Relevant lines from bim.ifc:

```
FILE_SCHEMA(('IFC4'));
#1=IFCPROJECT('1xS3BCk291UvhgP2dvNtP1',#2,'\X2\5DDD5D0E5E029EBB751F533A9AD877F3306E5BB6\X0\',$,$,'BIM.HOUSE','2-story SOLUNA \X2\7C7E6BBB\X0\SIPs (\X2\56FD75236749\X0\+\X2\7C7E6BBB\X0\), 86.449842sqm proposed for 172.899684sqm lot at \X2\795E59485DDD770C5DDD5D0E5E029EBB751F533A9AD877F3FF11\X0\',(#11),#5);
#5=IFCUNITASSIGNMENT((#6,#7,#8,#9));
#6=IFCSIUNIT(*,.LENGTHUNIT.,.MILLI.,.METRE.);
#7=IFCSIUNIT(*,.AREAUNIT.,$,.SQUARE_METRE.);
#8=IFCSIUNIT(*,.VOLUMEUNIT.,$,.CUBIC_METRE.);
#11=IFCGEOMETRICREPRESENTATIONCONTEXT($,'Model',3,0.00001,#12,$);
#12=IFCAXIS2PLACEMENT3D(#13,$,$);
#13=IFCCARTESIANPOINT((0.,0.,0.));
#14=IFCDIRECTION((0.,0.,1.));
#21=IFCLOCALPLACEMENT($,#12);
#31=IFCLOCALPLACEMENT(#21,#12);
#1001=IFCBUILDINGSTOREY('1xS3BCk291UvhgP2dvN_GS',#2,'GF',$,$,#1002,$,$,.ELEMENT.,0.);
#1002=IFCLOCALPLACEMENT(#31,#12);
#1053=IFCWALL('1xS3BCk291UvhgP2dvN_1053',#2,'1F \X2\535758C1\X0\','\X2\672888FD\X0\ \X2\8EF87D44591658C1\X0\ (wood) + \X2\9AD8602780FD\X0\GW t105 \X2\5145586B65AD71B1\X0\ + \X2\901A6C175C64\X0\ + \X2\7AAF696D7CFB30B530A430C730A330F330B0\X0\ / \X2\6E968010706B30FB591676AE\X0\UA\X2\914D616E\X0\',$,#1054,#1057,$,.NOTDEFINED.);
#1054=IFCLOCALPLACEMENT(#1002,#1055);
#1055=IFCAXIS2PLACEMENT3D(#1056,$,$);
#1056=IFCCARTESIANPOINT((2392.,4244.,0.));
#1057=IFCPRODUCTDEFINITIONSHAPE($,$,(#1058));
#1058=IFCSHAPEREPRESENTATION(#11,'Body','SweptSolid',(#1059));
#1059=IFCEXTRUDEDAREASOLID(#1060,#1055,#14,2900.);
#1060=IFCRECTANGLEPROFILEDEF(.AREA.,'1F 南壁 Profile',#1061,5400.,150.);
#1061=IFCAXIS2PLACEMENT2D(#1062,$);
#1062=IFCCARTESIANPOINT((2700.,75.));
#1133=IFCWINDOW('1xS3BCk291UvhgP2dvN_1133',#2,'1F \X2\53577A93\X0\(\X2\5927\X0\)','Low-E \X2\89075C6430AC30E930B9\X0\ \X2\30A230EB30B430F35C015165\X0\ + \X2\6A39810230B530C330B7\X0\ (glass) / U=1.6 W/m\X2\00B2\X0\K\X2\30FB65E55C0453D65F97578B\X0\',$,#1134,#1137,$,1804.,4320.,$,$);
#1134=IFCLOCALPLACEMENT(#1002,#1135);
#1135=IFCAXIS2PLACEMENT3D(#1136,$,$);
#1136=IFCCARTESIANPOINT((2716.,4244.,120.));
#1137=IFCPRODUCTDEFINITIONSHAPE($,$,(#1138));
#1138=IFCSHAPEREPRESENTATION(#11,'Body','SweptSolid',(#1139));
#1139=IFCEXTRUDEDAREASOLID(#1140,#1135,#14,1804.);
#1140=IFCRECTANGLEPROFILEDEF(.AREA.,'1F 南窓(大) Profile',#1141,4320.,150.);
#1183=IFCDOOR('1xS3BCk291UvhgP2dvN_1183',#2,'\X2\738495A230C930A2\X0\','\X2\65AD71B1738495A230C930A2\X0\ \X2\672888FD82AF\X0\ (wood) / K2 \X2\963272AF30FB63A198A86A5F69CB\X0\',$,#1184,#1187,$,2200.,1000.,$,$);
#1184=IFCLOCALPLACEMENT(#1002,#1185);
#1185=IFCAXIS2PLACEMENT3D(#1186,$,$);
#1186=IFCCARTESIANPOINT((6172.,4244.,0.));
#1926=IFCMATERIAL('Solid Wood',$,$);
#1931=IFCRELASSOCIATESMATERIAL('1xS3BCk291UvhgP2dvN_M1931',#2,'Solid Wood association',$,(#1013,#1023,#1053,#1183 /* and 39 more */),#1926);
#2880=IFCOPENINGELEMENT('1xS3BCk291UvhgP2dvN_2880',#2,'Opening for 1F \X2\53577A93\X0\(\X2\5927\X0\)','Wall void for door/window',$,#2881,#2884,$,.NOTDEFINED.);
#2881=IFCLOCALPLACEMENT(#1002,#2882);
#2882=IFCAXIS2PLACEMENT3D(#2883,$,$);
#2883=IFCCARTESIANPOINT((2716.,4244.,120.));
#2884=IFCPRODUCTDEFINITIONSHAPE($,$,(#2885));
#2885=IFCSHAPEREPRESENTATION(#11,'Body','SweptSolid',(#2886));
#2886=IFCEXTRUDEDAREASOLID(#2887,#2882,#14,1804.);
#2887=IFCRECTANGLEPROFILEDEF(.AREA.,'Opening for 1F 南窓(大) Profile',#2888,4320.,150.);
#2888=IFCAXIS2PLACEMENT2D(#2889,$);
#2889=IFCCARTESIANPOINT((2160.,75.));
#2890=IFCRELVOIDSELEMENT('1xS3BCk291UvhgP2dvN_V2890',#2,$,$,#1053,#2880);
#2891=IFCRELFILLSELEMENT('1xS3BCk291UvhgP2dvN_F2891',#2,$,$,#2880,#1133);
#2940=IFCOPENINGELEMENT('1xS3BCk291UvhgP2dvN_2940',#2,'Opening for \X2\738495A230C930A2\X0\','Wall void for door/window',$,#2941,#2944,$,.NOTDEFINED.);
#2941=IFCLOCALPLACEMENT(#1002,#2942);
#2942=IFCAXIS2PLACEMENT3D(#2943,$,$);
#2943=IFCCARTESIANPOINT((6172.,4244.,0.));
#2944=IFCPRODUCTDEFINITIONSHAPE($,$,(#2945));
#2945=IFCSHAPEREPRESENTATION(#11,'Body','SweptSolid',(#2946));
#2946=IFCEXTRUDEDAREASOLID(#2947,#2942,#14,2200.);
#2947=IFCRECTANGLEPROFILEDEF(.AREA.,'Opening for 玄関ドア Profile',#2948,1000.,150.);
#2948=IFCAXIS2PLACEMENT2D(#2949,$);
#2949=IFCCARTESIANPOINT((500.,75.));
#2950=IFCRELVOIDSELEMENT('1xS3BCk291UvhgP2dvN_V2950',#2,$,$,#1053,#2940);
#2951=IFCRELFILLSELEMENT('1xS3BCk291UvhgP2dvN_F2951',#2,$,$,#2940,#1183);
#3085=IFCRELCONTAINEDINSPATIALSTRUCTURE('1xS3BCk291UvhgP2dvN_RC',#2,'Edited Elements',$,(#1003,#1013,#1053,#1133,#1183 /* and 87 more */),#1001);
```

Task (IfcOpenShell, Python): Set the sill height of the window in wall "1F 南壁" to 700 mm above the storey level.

```python
import numpy as np
import ifcopenshell
import ifcopenshell.api.geometry
import ifcopenshell.geom
import ifcopenshell.util.element
import ifcopenshell.util.placement
import ifcopenshell.util.shape
import ifcopenshell.util.unit

model = ifcopenshell.open("bim.ifc")
unit_scale = ifcopenshell.util.unit.calculate_unit_scale(model)

window = model.by_id(1133)
opening = window.FillsVoids[0].RelatingOpeningElement
storey = ifcopenshell.util.element.get_container(window, ifc_class="IfcBuildingStorey")
level = ifcopenshell.util.placement.get_local_placement(storey.ObjectPlacement)[2, 3]

# The opening's origin need not be at the sill, so measure its lowest point.
shape = ifcopenshell.geom.create_shape(ifcopenshell.geom.settings(), opening)
bottom = ifcopenshell.util.shape.get_shape_bottom_elevation(shape, shape.geometry) / unit_scale
dz = level + 0.7 / unit_scale - bottom

shift = np.array([0.0, 0.0, dz])
# The window is not placed relative to its opening, so move both.
for product in (opening, window):
    matrix = ifcopenshell.util.placement.get_local_placement(product.ObjectPlacement)
    matrix[:3, 3] += shift
    ifcopenshell.api.geometry.edit_object_placement(model, product=product, matrix=matrix, is_si=False)

print(f"moved by {dz * unit_scale:+.3f} m")

model.write("bim-out.ifc")
```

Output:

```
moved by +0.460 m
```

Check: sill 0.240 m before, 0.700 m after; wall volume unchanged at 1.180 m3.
